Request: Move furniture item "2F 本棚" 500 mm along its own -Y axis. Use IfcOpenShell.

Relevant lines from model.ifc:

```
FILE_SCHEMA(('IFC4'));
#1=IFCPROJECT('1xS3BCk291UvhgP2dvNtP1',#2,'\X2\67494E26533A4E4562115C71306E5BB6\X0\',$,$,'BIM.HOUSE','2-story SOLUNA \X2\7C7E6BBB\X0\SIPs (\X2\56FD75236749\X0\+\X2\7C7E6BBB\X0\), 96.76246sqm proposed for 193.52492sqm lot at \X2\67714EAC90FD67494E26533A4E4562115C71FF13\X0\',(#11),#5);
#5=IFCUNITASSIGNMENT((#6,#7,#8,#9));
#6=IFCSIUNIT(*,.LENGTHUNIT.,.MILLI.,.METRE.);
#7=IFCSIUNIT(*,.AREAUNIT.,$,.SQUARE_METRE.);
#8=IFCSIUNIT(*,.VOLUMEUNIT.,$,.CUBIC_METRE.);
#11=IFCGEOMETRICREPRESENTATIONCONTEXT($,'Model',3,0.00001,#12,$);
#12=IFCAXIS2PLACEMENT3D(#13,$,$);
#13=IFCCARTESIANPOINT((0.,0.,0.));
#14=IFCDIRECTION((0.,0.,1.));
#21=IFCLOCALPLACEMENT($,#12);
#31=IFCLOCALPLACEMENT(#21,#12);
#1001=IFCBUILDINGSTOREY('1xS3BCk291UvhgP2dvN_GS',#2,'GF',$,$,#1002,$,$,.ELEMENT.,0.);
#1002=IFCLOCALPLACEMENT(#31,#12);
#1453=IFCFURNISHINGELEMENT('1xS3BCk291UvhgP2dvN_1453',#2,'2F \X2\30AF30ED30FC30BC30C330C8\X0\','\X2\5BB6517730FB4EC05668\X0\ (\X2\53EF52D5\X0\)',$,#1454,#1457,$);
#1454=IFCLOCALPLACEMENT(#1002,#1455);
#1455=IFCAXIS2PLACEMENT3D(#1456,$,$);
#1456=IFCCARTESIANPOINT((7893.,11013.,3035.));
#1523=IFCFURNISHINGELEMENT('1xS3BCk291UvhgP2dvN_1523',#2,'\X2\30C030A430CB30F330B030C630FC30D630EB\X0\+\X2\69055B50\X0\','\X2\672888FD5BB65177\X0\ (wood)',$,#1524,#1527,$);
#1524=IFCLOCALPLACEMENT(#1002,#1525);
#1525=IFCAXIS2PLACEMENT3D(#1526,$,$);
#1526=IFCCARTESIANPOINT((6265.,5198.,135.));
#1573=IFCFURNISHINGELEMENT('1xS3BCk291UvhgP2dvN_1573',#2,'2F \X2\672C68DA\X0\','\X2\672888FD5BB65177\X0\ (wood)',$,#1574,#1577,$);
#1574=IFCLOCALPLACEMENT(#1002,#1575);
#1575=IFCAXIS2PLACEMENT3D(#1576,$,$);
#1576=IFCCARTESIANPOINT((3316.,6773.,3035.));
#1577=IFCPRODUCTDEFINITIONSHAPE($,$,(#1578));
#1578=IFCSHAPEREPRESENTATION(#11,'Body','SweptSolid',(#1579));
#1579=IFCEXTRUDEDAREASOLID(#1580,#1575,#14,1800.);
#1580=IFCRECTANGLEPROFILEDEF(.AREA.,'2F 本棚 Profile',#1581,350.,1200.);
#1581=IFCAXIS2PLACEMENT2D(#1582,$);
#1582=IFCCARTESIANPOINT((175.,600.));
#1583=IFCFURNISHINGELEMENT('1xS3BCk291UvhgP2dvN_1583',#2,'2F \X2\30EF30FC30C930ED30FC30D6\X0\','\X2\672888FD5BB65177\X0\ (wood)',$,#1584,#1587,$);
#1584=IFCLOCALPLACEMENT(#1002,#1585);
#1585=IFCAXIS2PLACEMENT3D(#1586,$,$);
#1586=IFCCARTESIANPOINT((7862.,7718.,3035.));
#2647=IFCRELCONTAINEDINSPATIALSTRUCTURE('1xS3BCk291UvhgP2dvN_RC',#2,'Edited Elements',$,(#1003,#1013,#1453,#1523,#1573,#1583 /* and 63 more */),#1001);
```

```python
import ifcopenshell
import ifcopenshell.api.geometry
import ifcopenshell.util.placement

model = ifcopenshell.open("model.ifc")

item = model.by_guid("1xS3BCk291UvhgP2dvN_1573")
matrix = ifcopenshell.util.placement.get_local_placement(item.ObjectPlacement)
matrix[:3, 3] -= matrix[:3, 1] * 500.0
ifcopenshell.api.geometry.edit_object_placement(model, product=item, matrix=matrix, is_si=False)

print(ifcopenshell.util.placement.get_local_placement(item.ObjectPlacement).round(3) + 0.0)

model.write("model_v2.ifc")
```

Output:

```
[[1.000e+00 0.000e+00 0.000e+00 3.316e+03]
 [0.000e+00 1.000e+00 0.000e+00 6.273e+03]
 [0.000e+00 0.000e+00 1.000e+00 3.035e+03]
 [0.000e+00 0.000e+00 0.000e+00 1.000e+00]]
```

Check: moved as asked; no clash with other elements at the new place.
